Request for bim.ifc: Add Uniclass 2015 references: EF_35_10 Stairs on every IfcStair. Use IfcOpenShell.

First a look at what the model holds.

```python
import ifcopenshell

model = ifcopenshell.open("bim.ifc")
print(model.schema)
print("classifications:", [c.Name for c in model.by_type("IfcClassification")])
for ifc_class in ("IfcDoor", "IfcRoof", "IfcStair", "IfcWall", "IfcWindow"):
    print(ifc_class, len(model.by_type(ifc_class)))
```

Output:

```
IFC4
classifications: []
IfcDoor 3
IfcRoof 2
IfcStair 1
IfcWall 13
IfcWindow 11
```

```python
import ifcopenshell
import ifcopenshell.api.classification

model = ifcopenshell.open("bim.ifc")

system = ifcopenshell.api.classification.add_classification(model, classification="Uniclass 2015")

codes = {
    "IfcStair": ("EF_35_10", "Stairs"),
}
for ifc_class, (code, name) in codes.items():
    products = model.by_type(ifc_class)
    ifcopenshell.api.classification.add_reference(
        model, products=products, classification=system, identification=code, name=name
    )
    print(code, len(products))

model.write("bim_v2.ifc")
```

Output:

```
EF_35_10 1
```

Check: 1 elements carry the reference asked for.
